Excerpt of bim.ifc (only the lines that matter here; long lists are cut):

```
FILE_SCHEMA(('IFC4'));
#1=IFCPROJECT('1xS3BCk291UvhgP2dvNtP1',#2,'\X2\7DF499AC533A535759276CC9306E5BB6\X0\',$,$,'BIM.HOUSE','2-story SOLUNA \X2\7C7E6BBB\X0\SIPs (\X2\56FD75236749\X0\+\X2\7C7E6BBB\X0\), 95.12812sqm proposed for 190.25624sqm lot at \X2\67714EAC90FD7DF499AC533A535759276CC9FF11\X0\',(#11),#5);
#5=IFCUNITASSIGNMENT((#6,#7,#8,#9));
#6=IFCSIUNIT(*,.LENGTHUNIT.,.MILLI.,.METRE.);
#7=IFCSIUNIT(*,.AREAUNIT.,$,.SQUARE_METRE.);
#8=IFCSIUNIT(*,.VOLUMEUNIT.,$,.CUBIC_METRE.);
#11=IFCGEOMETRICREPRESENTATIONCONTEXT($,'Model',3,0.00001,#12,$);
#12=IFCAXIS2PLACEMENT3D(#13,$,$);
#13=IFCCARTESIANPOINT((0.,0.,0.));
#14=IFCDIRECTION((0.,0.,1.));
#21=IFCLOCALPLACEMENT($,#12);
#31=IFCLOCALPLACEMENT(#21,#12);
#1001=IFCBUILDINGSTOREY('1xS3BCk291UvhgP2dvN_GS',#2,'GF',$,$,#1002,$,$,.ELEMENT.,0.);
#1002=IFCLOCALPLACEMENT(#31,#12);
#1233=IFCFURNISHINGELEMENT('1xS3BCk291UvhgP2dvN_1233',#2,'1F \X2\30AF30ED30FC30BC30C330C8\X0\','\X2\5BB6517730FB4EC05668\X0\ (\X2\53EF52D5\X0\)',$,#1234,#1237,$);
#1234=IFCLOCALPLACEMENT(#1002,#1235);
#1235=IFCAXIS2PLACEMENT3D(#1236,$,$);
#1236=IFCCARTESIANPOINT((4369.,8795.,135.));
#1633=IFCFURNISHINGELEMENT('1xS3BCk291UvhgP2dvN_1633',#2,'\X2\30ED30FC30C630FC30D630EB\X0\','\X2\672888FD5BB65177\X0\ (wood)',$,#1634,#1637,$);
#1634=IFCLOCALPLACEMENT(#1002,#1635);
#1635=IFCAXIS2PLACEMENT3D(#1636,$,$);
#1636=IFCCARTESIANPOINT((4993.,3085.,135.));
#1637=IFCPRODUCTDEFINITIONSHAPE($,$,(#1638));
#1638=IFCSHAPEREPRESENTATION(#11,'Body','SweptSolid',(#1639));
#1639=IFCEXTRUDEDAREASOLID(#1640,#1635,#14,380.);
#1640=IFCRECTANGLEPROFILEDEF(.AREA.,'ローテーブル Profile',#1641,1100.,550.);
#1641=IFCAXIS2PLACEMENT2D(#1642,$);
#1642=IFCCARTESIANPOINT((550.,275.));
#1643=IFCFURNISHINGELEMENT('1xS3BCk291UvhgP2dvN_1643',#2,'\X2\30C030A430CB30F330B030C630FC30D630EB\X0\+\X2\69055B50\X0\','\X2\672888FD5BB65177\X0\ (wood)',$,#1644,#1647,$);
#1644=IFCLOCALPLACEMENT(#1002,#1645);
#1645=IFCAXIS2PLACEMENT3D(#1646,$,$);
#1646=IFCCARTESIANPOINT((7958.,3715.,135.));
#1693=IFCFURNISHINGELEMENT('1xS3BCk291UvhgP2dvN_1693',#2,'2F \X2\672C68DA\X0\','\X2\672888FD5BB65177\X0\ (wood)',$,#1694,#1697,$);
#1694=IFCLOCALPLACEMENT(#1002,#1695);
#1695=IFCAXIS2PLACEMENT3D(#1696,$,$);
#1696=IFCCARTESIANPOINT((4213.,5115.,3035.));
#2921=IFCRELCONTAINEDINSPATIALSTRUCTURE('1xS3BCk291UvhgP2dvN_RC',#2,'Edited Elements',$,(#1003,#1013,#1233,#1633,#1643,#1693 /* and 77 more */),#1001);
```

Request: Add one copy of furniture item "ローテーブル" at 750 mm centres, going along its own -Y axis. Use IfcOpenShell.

```python
import ifcopenshell
import ifcopenshell.api.geometry
import ifcopenshell.api.root
import ifcopenshell.util.element
import ifcopenshell.util.placement

model = ifcopenshell.open("bim.ifc")


def reuse_history(source, copy):
    """copy_class also copies each property set's owner history, people and application; keep the originals."""
    for rel in copy.IsDefinedBy:
        if rel.is_a("IfcRelDefinesByProperties") and (history := rel.RelatingPropertyDefinition.OwnerHistory):
            rel.RelatingPropertyDefinition.OwnerHistory = source.OwnerHistory
            ifcopenshell.util.element.remove_deep2(model, history)


source = model.by_guid("1xS3BCk291UvhgP2dvN_1633")
base = ifcopenshell.util.placement.get_local_placement(source.ObjectPlacement)
step = -base[:3, 1] * 750.0

for i in range(1, 2):
    copy = ifcopenshell.api.root.copy_class(model, product=source)
    copy.Representation = ifcopenshell.util.element.copy_deep(
        model, source.Representation, exclude=["IfcGeometricRepresentationContext", "IfcRepresentationMap"]
    )
    reuse_history(source, copy)
    matrix = base.copy()
    matrix[:3, 3] += i * step
    print("added at", matrix[:3, 3].round(3) + 0.0)
    ifcopenshell.api.geometry.edit_object_placement(model, product=copy, matrix=matrix, is_si=False)

model.write("bim-out.ifc")
```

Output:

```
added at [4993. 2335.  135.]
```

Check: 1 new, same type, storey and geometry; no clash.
